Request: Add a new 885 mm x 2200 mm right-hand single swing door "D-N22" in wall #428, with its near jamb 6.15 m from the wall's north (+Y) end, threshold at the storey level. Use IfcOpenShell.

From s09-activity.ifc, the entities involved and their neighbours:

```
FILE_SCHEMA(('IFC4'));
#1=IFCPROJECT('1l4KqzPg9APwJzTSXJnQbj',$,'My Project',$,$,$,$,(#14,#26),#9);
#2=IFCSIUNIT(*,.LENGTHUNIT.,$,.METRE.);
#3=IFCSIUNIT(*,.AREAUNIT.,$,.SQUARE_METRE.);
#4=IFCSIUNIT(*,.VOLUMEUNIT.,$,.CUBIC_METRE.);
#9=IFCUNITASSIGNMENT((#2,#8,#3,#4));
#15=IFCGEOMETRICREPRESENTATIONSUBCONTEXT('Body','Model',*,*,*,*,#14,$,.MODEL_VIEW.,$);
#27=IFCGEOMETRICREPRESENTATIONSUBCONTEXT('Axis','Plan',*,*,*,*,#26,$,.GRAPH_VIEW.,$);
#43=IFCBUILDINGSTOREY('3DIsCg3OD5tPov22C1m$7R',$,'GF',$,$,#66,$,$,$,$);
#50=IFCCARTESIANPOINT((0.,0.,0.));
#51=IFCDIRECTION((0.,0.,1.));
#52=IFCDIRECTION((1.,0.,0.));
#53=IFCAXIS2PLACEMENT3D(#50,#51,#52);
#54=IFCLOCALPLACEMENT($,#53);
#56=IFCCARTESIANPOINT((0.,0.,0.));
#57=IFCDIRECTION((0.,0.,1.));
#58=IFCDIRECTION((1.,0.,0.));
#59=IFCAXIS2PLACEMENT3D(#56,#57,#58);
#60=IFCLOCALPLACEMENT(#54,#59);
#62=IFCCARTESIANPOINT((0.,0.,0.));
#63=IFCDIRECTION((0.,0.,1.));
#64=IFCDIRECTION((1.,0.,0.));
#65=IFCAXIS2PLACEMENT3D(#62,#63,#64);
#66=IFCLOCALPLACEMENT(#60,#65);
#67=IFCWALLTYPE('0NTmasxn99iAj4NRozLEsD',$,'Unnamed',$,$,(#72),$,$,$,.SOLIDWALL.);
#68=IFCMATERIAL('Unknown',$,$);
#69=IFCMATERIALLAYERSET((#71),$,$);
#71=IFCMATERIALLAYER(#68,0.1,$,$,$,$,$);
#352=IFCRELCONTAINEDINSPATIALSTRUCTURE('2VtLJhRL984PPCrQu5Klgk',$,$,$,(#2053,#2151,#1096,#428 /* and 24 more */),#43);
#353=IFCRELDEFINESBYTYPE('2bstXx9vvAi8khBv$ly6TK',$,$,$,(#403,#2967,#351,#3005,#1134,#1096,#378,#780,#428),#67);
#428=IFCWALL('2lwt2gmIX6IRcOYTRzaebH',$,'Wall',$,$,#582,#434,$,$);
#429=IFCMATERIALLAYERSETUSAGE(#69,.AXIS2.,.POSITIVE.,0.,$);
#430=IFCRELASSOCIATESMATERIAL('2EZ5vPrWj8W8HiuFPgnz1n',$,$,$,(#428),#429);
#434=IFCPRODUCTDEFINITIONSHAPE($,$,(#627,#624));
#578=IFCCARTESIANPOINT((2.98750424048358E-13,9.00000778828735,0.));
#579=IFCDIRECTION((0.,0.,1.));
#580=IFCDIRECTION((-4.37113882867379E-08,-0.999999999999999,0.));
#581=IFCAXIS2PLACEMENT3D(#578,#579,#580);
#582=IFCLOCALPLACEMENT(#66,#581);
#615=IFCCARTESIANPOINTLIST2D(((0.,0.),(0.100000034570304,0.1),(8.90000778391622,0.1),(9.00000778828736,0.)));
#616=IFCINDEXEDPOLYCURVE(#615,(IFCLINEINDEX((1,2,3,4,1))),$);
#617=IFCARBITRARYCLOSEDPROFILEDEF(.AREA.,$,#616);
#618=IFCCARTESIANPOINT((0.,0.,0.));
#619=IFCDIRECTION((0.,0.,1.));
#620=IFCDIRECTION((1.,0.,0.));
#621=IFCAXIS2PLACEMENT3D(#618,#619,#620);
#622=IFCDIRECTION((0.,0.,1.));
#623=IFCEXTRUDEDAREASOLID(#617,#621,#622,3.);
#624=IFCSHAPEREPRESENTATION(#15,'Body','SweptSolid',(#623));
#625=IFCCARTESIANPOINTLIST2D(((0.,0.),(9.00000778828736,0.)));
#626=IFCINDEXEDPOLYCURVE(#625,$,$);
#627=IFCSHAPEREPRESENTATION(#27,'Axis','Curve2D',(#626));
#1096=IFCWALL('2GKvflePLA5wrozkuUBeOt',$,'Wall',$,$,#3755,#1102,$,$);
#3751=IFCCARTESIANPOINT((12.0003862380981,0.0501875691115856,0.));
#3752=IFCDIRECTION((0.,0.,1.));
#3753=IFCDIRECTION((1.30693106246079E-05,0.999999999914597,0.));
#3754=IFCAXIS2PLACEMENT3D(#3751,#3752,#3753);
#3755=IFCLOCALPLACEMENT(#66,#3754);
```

```python
import numpy as np
import ifcopenshell
import ifcopenshell.api.feature
import ifcopenshell.api.geometry
import ifcopenshell.api.root
import ifcopenshell.api.spatial
import ifcopenshell.geom
import ifcopenshell.util.element
import ifcopenshell.util.placement
import ifcopenshell.util.representation
import ifcopenshell.util.shape
import ifcopenshell.util.unit

model = ifcopenshell.open("s09-activity.ifc")
unit_scale = ifcopenshell.util.unit.calculate_unit_scale(model)
settings = ifcopenshell.geom.settings()


def volume(element):
    """Net volume in cubic metres, openings subtracted."""
    shape = ifcopenshell.geom.create_shape(settings, element)
    return ifcopenshell.util.shape.get_volume(shape.geometry)


wall = model.by_guid("2lwt2gmIX6IRcOYTRzaebH")
storey = ifcopenshell.util.element.get_container(wall, ifc_class="IfcBuildingStorey")
context = ifcopenshell.util.representation.get_context(model, "Model", "Body", "MODEL_VIEW")
before = volume(wall)

width, height, from_end, sill = 0.885, 2.2, 6.15, 0.0  # metres

# The wall runs along its own X axis, and the end named is its -X end.
wall_shape = ifcopenshell.geom.create_shape(settings, wall)
x, y, z = ifcopenshell.util.shape.get_vertices(wall_shape.geometry).T
start = x.min() + from_end
face, thickness = float(y.min()), float(y.max() - y.min())
wall_matrix = ifcopenshell.util.placement.get_local_placement(wall.ObjectPlacement)
level = ifcopenshell.util.placement.get_local_placement(storey.ObjectPlacement)[2, 3]


def in_wall(x, y):
    """Placement at x, y metres in the wall's axes, at sill height."""
    matrix = wall_matrix.copy()
    matrix[:, 3] = wall_matrix @ np.array([x / unit_scale, y / unit_scale, 0.0, 1.0])
    matrix[2, 3] = level + sill / unit_scale
    return matrix


# Opening: a box that overshoots both wall faces by 50 mm.
opening = ifcopenshell.api.root.create_entity(model, ifc_class="IfcOpeningElement", predefined_type="OPENING")
box = ifcopenshell.api.geometry.add_wall_representation(
    model, context=context, length=width, height=height, thickness=thickness + 0.1
)
ifcopenshell.api.geometry.assign_representation(model, product=opening, representation=box)
ifcopenshell.api.geometry.edit_object_placement(model, product=opening, matrix=in_wall(start, face - 0.05), is_si=False)
ifcopenshell.api.feature.add_feature(model, feature=opening, element=wall)

door = ifcopenshell.api.root.create_entity(model, ifc_class="IfcDoor", name="D-N22", predefined_type="DOOR")
door.OverallWidth, door.OverallHeight = width / unit_scale, height / unit_scale
door.OperationType = "SINGLE_SWING_RIGHT"
body = ifcopenshell.api.geometry.add_door_representation(
    model,
    context=context,
    overall_width=door.OverallWidth,
    overall_height=door.OverallHeight,
    operation_type="SINGLE_SWING_RIGHT",
    lining_properties={"LiningDepth": thickness / unit_scale, "ThresholdDepth": thickness / unit_scale},
)
ifcopenshell.api.geometry.assign_representation(model, product=door, representation=body)
ifcopenshell.api.spatial.assign_container(model, products=[door], relating_structure=storey)
ifcopenshell.api.feature.add_filling(model, opening=opening, element=door)

# The lining spans the wall, so the door starts at the wall face.
ifcopenshell.api.geometry.edit_object_placement(model, product=door, matrix=in_wall(start, face), is_si=False)

after = volume(wall)

print(f"wall volume {before:.3f} -> {after:.3f} m3")

model.write("s09-activity_v2.ifc")
```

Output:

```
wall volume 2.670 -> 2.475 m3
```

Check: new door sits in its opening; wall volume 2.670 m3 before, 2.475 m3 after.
